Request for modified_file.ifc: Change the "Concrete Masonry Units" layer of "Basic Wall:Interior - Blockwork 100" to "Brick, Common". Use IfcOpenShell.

First a look at what the model holds.

```python
import ifcopenshell
import ifcopenshell.util.element

model = ifcopenshell.open("modified_file.ifc")
print(model.schema)
for layer_set in model.by_type("IfcMaterialLayerSet"):
    if layer_set.LayerSetName == "Basic Wall:Interior - Blockwork 100":
        for layer in layer_set.MaterialLayers:
            print(layer.id(), layer.Material and layer.Material.Name, layer.LayerThickness, sep=" | ")
        print(len(ifcopenshell.util.element.get_elements_by_material(model, layer_set)), "elements and types use it")
print(sorted(m.Name for m in model.by_type("IfcMaterial") if m.Name)[:60])
```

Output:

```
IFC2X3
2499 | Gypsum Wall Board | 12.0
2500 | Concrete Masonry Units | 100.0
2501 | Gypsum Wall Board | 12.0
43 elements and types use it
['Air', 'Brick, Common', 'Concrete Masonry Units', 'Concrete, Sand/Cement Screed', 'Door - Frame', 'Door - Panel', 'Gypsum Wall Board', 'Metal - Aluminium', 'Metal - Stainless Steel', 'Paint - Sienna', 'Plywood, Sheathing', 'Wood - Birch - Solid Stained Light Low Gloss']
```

```python
import ifcopenshell
import ifcopenshell.api.material

model = ifcopenshell.open("modified_file.ifc")

layer_set = next(s for s in model.by_type("IfcMaterialLayerSet") if s.LayerSetName == "Basic Wall:Interior - Blockwork 100")
layer = next(l for l in layer_set.MaterialLayers if l.Material and l.Material.Name == "Concrete Masonry Units")
material = next(m for m in model.by_type("IfcMaterial") if m.Name == "Brick, Common")

# Point this one layer at the other material; renaming the old one would change it everywhere.
ifcopenshell.api.material.edit_layer(model, layer=layer, attributes={}, material=material)

print([l.Material.Name if l.Material else None for l in layer_set.MaterialLayers])

model.write("modified_file_rev.ifc")
```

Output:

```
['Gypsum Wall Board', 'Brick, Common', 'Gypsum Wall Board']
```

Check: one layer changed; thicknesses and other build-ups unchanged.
